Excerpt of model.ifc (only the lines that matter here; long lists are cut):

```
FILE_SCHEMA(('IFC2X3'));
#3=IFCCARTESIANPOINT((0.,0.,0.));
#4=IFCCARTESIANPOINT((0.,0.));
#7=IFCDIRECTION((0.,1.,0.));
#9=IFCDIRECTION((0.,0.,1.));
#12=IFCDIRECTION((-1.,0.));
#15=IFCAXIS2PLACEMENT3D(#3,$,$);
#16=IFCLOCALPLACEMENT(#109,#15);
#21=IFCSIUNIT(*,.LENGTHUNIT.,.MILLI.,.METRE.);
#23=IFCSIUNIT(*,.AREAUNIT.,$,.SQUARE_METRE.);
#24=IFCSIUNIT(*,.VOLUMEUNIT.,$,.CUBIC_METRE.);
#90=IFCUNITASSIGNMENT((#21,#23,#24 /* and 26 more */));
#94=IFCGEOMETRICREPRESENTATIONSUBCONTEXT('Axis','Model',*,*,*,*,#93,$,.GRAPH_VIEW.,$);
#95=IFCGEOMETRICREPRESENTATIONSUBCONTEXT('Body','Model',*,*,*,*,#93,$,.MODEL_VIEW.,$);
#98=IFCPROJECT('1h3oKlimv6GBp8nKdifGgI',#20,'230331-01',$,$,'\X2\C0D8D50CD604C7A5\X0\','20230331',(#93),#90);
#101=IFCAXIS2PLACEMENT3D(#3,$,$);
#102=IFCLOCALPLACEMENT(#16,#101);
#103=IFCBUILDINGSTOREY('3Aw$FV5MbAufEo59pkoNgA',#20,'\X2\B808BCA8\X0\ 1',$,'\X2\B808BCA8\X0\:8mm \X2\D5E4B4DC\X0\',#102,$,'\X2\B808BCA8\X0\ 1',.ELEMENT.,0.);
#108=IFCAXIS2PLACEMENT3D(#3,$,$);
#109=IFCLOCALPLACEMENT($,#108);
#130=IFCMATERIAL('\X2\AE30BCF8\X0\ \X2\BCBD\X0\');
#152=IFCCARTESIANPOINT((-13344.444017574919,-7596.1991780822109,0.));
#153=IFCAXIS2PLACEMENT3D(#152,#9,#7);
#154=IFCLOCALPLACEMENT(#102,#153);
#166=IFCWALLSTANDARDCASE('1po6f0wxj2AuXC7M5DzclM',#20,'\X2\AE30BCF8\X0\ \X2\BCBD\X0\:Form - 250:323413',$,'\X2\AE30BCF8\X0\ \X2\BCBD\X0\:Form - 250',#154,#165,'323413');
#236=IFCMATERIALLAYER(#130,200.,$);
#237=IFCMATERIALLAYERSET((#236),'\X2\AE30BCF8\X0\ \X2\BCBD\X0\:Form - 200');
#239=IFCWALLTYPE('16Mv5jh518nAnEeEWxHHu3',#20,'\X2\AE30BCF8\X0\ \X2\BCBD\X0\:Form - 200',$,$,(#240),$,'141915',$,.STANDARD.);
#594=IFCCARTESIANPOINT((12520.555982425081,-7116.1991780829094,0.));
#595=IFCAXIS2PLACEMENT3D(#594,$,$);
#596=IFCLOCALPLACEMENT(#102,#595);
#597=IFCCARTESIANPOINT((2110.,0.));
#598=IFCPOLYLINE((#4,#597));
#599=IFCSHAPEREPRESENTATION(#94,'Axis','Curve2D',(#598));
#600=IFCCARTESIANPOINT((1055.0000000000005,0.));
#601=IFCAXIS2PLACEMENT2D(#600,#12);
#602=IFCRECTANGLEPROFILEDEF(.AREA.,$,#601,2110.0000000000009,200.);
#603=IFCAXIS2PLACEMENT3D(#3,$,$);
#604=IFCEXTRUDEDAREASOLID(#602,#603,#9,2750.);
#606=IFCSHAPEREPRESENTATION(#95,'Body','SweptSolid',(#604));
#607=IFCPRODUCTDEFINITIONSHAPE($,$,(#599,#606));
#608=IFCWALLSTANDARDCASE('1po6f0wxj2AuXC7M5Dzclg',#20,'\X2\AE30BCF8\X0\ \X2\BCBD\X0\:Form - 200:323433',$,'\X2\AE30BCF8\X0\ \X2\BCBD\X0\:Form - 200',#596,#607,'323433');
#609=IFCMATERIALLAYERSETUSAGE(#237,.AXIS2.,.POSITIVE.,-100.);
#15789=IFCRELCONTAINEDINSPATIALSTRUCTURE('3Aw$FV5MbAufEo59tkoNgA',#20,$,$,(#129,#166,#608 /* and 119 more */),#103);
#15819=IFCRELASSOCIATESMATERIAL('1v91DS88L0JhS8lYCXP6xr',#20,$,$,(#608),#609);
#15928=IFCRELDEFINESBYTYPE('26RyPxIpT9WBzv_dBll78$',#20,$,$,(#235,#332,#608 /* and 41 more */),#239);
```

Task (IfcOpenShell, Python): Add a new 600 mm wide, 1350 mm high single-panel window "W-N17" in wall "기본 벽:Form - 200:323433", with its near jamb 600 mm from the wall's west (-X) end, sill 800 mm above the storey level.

```python
import numpy as np
import ifcopenshell
import ifcopenshell.api.feature
import ifcopenshell.api.geometry
import ifcopenshell.api.root
import ifcopenshell.api.spatial
import ifcopenshell.api.type
import ifcopenshell.geom
import ifcopenshell.util.element
import ifcopenshell.util.placement
import ifcopenshell.util.representation
import ifcopenshell.util.shape
import ifcopenshell.util.unit

model = ifcopenshell.open("model.ifc")
unit_scale = ifcopenshell.util.unit.calculate_unit_scale(model)
settings = ifcopenshell.geom.settings()


def volume(element):
    """Net volume in cubic metres, openings subtracted."""
    shape = ifcopenshell.geom.create_shape(settings, element)
    return ifcopenshell.util.shape.get_volume(shape.geometry)


wall = model.by_guid("1po6f0wxj2AuXC7M5Dzclg")
storey = ifcopenshell.util.element.get_container(wall, ifc_class="IfcBuildingStorey")
context = ifcopenshell.util.representation.get_context(model, "Model", "Body", "MODEL_VIEW")
before = volume(wall)

width, height, from_end, sill = 0.6, 1.35, 0.6, 0.8  # metres

# The wall runs along its own X axis, and the end named is its -X end.
wall_shape = ifcopenshell.geom.create_shape(settings, wall)
x, y, z = ifcopenshell.util.shape.get_vertices(wall_shape.geometry).T
start = x.min() + from_end
face, thickness = float(y.min()), float(y.max() - y.min())
wall_matrix = ifcopenshell.util.placement.get_local_placement(wall.ObjectPlacement)
level = ifcopenshell.util.placement.get_local_placement(storey.ObjectPlacement)[2, 3]


def in_wall(x, y):
    """Placement at x, y metres in the wall's axes, at sill height."""
    matrix = wall_matrix.copy()
    matrix[:, 3] = wall_matrix @ np.array([x / unit_scale, y / unit_scale, 0.0, 1.0])
    matrix[2, 3] = level + sill / unit_scale
    return matrix


# Opening: a box that overshoots both wall faces by 50 mm.
opening = ifcopenshell.api.root.create_entity(model, ifc_class="IfcOpeningElement")
box = ifcopenshell.api.geometry.add_wall_representation(
    model, context=context, length=width, height=height, thickness=thickness + 0.1
)
ifcopenshell.api.geometry.assign_representation(model, product=opening, representation=box)
ifcopenshell.api.geometry.edit_object_placement(model, product=opening, matrix=in_wall(start, face - 0.05), is_si=False)
ifcopenshell.api.feature.add_feature(model, feature=opening, element=wall)

window = ifcopenshell.api.root.create_entity(model, ifc_class="IfcWindow", name="W-N17")
window.OverallWidth, window.OverallHeight = width / unit_scale, height / unit_scale
body = ifcopenshell.api.geometry.add_window_representation(
    model,
    context=context,
    overall_width=window.OverallWidth,
    overall_height=window.OverallHeight,
    partition_type="SINGLE_PANEL",
)
ifcopenshell.api.geometry.assign_representation(model, product=window, representation=body)
ifcopenshell.api.spatial.assign_container(model, products=[window], relating_structure=storey)
fills = ifcopenshell.api.feature.add_filling(model, opening=opening, element=window)
fills.OwnerHistory = window.OwnerHistory  # required in IFC2X3

# IFC2X3 keeps the operation on the window style.
style = ifcopenshell.api.root.create_entity(model, ifc_class="IfcWindowStyle", name="W-N17")
style.OperationType, style.ConstructionType = "SINGLE_PANEL", "NOTDEFINED"
style.ParameterTakesPrecedence = style.Sizeable = False
ifcopenshell.api.type.assign_type(model, related_objects=[window], relating_type=style)

# Centre the window in the wall's thickness.
ifcopenshell.api.geometry.edit_object_placement(model, product=window, matrix=in_wall(start, face), is_si=False)
window_shape = ifcopenshell.geom.create_shape(settings, window)
depth = ifcopenshell.util.shape.get_vertices(window_shape.geometry)[:, 1]
offset = face + thickness / 2 - (depth.min() + depth.max()) / 2
ifcopenshell.api.geometry.edit_object_placement(model, product=window, matrix=in_wall(start, offset), is_si=False)

after = volume(wall)

print(f"wall volume {before:.3f} -> {after:.3f} m3")

model.write("model_rev.ifc")
```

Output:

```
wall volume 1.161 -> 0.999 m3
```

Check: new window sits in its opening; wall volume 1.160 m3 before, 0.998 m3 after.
